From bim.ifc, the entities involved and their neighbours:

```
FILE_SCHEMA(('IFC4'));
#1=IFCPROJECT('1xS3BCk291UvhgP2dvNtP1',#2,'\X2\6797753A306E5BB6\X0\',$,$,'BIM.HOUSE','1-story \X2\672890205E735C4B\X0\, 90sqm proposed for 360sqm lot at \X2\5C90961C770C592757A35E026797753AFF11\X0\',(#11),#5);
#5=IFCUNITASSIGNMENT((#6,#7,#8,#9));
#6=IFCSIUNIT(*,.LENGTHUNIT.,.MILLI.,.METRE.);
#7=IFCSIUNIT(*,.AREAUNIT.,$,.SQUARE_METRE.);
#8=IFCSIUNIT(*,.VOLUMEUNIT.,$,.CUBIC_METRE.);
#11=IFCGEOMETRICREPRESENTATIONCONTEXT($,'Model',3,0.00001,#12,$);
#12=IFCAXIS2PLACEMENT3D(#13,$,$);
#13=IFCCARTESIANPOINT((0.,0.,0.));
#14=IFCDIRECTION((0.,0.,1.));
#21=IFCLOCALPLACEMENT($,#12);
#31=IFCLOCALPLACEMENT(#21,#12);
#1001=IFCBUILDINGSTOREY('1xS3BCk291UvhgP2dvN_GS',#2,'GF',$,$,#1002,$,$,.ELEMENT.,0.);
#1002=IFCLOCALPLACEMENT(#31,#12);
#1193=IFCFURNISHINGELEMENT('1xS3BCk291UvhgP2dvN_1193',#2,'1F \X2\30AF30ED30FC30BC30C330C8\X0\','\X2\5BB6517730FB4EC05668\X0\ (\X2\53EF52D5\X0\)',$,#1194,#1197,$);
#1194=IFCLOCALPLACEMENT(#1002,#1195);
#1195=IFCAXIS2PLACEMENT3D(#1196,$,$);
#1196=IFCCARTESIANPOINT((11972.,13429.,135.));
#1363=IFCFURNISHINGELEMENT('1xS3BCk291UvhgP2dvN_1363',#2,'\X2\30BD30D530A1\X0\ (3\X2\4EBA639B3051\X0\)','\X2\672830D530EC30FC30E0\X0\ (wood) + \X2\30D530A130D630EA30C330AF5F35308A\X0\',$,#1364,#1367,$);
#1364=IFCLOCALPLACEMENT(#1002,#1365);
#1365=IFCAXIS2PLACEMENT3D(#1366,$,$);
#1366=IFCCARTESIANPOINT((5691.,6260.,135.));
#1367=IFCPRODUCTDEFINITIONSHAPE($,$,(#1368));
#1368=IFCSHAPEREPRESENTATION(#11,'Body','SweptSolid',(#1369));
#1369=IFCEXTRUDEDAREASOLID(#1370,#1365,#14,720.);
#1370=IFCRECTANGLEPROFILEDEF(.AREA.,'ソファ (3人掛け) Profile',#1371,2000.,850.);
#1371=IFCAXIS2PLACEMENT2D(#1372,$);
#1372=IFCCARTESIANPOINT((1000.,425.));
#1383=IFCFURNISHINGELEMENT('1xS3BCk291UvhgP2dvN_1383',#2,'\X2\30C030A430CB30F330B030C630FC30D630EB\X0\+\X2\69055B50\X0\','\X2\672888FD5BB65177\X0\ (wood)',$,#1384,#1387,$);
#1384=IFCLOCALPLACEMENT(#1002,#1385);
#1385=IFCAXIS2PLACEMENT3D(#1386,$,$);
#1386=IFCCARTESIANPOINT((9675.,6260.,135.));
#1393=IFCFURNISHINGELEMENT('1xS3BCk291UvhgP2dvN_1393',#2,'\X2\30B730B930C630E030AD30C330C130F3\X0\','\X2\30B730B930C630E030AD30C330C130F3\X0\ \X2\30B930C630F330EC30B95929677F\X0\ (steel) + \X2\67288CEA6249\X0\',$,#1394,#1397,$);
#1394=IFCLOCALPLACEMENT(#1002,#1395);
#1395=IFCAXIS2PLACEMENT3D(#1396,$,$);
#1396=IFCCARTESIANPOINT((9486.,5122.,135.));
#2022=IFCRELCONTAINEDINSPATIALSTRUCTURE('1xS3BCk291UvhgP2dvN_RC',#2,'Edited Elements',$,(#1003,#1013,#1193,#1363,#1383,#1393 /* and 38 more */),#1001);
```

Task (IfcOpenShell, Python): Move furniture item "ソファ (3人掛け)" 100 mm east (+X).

```python
import ifcopenshell
import ifcopenshell.api.geometry
import ifcopenshell.util.placement

model = ifcopenshell.open("bim.ifc")

item = model.by_guid("1xS3BCk291UvhgP2dvN_1363")
matrix = ifcopenshell.util.placement.get_local_placement(item.ObjectPlacement)
matrix[0, 3] += 100.0
ifcopenshell.api.geometry.edit_object_placement(model, product=item, matrix=matrix, is_si=False)

print(ifcopenshell.util.placement.get_local_placement(item.ObjectPlacement).round(3) + 0.0)

model.write("bim_v2.ifc")
```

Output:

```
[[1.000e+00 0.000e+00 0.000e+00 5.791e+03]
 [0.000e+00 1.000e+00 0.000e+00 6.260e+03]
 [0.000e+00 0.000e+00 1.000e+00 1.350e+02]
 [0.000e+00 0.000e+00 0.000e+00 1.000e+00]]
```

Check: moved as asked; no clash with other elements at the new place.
